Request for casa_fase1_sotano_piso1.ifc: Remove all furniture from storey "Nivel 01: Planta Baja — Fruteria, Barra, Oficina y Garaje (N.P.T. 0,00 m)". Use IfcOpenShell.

First a look at what the model holds.

```python
import ifcopenshell
import ifcopenshell.util.element

model = ifcopenshell.open("casa_fase1_sotano_piso1.ifc")
print(model.schema)
storey = next(s for s in model.by_type("IfcBuildingStorey") if s.Name == "Nivel 01: Planta Baja — Fruteria, Barra, Oficina y Garaje (N.P.T. 0,00 m)")
furniture = [e for e in ifcopenshell.util.element.get_decomposition(storey) if e.is_a("IfcFurnishingElement")]
seen = {}
for e in furniture:
    element_type = ifcopenshell.util.element.get_type(e)
    name = element_type.Name if element_type not in (None, e) else None
    seen[name] = seen.get(name, 0) + 1
for name, count in sorted(seen.items(), key=str):
    print(count, "x", name)
```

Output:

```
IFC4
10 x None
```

```python
import ifcopenshell
import ifcopenshell.api.root
import ifcopenshell.util.element

model = ifcopenshell.open("casa_fase1_sotano_piso1.ifc")

storey = next(s for s in model.by_type("IfcBuildingStorey") if s.Name == "Nivel 01: Planta Baja — Fruteria, Barra, Oficina y Garaje (N.P.T. 0,00 m)")
furniture = [e for e in ifcopenshell.util.element.get_decomposition(storey) if e.is_a("IfcFurnishingElement")]

for e in furniture:
    ifcopenshell.api.root.remove_product(model, product=e)
print(len(furniture), "removed")

model.write("casa_fase1_sotano_piso1_edited.ifc")
```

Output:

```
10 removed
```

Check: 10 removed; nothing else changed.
